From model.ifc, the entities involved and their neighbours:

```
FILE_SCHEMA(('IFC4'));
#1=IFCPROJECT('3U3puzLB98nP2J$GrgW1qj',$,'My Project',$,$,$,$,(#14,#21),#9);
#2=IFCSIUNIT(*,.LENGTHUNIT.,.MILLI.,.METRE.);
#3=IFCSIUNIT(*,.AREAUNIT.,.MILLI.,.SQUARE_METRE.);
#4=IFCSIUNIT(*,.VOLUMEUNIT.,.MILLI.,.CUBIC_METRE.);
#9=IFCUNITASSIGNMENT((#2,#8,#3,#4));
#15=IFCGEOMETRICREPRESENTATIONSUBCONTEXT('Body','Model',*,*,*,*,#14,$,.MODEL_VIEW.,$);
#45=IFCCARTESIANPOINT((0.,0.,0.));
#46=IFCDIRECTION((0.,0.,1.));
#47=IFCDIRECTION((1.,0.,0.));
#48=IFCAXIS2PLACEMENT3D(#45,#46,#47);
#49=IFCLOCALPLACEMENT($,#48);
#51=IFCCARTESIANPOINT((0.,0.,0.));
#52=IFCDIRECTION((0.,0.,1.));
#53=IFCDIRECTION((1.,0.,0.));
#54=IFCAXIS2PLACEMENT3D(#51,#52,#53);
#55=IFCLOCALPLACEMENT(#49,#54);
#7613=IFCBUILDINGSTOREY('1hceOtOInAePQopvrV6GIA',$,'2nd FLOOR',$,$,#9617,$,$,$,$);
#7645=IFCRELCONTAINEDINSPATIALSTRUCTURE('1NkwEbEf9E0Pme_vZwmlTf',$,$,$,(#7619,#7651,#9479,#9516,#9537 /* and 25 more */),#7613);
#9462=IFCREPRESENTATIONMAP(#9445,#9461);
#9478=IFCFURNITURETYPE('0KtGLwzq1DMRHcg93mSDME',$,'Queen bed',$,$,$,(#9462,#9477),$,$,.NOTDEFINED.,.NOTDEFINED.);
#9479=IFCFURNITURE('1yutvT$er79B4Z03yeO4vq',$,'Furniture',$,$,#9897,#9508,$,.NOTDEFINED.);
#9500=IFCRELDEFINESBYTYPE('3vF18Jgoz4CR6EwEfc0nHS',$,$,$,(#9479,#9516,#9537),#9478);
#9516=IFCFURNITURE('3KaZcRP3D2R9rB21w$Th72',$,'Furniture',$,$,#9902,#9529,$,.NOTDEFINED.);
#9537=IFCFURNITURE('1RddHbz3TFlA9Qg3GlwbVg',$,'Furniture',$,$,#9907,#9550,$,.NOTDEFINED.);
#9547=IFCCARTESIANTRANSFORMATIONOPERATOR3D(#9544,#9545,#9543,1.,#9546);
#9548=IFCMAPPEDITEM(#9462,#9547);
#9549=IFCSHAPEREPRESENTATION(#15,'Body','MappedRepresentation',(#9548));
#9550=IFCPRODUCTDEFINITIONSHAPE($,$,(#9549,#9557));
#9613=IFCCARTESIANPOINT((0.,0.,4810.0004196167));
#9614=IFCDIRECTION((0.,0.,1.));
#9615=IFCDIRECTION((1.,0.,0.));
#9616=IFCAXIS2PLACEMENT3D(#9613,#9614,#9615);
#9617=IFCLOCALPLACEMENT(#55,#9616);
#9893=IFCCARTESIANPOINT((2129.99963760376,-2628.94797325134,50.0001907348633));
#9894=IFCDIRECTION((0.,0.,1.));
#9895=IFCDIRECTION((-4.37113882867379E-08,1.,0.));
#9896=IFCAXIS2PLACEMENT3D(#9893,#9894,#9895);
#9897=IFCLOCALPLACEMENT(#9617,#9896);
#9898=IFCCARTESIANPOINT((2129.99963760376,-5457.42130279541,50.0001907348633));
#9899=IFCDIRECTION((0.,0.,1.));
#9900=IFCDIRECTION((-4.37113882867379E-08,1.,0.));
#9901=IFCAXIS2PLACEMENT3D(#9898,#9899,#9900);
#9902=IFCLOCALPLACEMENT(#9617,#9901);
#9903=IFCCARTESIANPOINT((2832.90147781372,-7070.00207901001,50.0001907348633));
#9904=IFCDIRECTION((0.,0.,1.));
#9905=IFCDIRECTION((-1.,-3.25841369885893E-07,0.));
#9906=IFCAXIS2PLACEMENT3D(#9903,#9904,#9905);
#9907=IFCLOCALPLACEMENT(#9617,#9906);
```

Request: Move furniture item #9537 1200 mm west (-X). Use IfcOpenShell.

```python
import ifcopenshell
import ifcopenshell.api.geometry
import ifcopenshell.util.placement

model = ifcopenshell.open("model.ifc")

item = model.by_guid("1RddHbz3TFlA9Qg3GlwbVg")
matrix = ifcopenshell.util.placement.get_local_placement(item.ObjectPlacement)
matrix[0, 3] -= 1200.0
ifcopenshell.api.geometry.edit_object_placement(model, product=item, matrix=matrix, is_si=False)

print(ifcopenshell.util.placement.get_local_placement(item.ObjectPlacement).round(3) + 0.0)

model.write("model-out.ifc")
```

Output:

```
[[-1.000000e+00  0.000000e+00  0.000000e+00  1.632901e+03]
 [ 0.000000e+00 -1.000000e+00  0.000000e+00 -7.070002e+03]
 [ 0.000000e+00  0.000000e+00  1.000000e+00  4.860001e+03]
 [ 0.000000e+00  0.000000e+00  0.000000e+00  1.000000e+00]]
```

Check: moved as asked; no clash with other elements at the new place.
